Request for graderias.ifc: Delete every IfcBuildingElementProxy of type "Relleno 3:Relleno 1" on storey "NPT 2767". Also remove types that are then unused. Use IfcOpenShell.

First a look at what the model holds.

```python
import ifcopenshell
import ifcopenshell.util.element

model = ifcopenshell.open("graderias.ifc")
print(model.schema)
storey = next(s for s in model.by_type("IfcBuildingStorey") if s.Name == "NPT 2767")
proxies = [e for e in ifcopenshell.util.element.get_decomposition(storey) if e.is_a("IfcBuildingElementProxy")]
seen = {}
for e in proxies:
    element_type = ifcopenshell.util.element.get_type(e)
    name = element_type.Name if element_type not in (None, e) else None
    seen[name] = seen.get(name, 0) + 1
for name, count in sorted(seen.items(), key=str):
    print(count, "x", name)
```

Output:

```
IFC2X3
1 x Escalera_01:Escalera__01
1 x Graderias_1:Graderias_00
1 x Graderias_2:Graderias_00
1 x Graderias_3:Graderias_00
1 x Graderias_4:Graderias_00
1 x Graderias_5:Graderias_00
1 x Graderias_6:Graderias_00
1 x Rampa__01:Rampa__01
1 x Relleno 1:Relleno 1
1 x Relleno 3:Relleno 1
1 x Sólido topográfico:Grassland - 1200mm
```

```python
import ifcopenshell
import ifcopenshell.api.root
import ifcopenshell.util.element

model = ifcopenshell.open("graderias.ifc")

storey = next(s for s in model.by_type("IfcBuildingStorey") if s.Name == "NPT 2767")
proxies = [e for e in ifcopenshell.util.element.get_decomposition(storey) if e.is_a("IfcBuildingElementProxy")]
targets = [e for e in proxies if (t := ifcopenshell.util.element.get_type(e)) not in (None, e) and t.Name == "Relleno 3:Relleno 1"]
types = {ifcopenshell.util.element.get_type(e) for e in targets} - {None, *targets}

for e in targets:
    ifcopenshell.api.root.remove_product(model, product=e)
print(len(targets), "removed")

unused = [t for t in types if not ifcopenshell.util.element.get_types(t)]
for t in unused:
    ifcopenshell.api.root.remove_product(model, product=t)
print(len(unused), "unused types removed")

model.write("graderias-out.ifc")
```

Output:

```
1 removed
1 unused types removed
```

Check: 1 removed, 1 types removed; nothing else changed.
